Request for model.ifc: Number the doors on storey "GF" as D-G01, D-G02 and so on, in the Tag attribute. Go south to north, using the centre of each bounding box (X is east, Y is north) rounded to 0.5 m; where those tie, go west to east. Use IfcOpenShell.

First a look at what the model holds.

```python
import ifcopenshell
import ifcopenshell.util.element
import ifcopenshell.util.placement

model = ifcopenshell.open("model.ifc")
print(model.schema)
storey = next(s for s in model.by_type("IfcBuildingStorey") if s.Name == "GF")
doors = [e for e in ifcopenshell.util.element.get_decomposition(storey) if e.is_a("IfcDoor")]
for e in sorted(doors, key=lambda e: e.id()):
    origin = ifcopenshell.util.placement.get_local_placement(e.ObjectPlacement)[:3, 3]
    print(e.id(), e.Tag, e.Name, origin.round(2) + 0.0, sep=" | ")
```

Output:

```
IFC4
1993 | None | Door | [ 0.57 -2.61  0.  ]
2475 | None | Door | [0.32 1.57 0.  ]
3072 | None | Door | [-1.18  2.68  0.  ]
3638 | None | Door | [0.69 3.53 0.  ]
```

```python
import ifcopenshell
import ifcopenshell.geom
import ifcopenshell.util.element
import ifcopenshell.util.shape

model = ifcopenshell.open("model.ifc")
settings = ifcopenshell.geom.settings()
settings.set("use-world-coords", True)


def centre(element):
    shape = ifcopenshell.geom.create_shape(settings, element)
    return ifcopenshell.util.shape.get_bbox_centroid(shape.geometry)


storey = next(s for s in model.by_type("IfcBuildingStorey") if s.Name == "GF")
doors = [e for e in ifcopenshell.util.element.get_decomposition(storey) if e.is_a("IfcDoor")]

# Insertion points can sit at a corner or the storey origin, so sort by the geometry (in metres).
centres = {e: centre(e) for e in doors}
doors.sort(key=lambda e: (round(centres[e][1] / 0.5), centres[e][0]))

for i, e in enumerate(doors, start=1):
    number = f"D-G{i:02d}"
    e.Tag = number
    print(e.id(), number)

model.write("model_updated.ifc")
```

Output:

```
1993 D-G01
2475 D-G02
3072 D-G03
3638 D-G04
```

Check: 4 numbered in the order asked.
